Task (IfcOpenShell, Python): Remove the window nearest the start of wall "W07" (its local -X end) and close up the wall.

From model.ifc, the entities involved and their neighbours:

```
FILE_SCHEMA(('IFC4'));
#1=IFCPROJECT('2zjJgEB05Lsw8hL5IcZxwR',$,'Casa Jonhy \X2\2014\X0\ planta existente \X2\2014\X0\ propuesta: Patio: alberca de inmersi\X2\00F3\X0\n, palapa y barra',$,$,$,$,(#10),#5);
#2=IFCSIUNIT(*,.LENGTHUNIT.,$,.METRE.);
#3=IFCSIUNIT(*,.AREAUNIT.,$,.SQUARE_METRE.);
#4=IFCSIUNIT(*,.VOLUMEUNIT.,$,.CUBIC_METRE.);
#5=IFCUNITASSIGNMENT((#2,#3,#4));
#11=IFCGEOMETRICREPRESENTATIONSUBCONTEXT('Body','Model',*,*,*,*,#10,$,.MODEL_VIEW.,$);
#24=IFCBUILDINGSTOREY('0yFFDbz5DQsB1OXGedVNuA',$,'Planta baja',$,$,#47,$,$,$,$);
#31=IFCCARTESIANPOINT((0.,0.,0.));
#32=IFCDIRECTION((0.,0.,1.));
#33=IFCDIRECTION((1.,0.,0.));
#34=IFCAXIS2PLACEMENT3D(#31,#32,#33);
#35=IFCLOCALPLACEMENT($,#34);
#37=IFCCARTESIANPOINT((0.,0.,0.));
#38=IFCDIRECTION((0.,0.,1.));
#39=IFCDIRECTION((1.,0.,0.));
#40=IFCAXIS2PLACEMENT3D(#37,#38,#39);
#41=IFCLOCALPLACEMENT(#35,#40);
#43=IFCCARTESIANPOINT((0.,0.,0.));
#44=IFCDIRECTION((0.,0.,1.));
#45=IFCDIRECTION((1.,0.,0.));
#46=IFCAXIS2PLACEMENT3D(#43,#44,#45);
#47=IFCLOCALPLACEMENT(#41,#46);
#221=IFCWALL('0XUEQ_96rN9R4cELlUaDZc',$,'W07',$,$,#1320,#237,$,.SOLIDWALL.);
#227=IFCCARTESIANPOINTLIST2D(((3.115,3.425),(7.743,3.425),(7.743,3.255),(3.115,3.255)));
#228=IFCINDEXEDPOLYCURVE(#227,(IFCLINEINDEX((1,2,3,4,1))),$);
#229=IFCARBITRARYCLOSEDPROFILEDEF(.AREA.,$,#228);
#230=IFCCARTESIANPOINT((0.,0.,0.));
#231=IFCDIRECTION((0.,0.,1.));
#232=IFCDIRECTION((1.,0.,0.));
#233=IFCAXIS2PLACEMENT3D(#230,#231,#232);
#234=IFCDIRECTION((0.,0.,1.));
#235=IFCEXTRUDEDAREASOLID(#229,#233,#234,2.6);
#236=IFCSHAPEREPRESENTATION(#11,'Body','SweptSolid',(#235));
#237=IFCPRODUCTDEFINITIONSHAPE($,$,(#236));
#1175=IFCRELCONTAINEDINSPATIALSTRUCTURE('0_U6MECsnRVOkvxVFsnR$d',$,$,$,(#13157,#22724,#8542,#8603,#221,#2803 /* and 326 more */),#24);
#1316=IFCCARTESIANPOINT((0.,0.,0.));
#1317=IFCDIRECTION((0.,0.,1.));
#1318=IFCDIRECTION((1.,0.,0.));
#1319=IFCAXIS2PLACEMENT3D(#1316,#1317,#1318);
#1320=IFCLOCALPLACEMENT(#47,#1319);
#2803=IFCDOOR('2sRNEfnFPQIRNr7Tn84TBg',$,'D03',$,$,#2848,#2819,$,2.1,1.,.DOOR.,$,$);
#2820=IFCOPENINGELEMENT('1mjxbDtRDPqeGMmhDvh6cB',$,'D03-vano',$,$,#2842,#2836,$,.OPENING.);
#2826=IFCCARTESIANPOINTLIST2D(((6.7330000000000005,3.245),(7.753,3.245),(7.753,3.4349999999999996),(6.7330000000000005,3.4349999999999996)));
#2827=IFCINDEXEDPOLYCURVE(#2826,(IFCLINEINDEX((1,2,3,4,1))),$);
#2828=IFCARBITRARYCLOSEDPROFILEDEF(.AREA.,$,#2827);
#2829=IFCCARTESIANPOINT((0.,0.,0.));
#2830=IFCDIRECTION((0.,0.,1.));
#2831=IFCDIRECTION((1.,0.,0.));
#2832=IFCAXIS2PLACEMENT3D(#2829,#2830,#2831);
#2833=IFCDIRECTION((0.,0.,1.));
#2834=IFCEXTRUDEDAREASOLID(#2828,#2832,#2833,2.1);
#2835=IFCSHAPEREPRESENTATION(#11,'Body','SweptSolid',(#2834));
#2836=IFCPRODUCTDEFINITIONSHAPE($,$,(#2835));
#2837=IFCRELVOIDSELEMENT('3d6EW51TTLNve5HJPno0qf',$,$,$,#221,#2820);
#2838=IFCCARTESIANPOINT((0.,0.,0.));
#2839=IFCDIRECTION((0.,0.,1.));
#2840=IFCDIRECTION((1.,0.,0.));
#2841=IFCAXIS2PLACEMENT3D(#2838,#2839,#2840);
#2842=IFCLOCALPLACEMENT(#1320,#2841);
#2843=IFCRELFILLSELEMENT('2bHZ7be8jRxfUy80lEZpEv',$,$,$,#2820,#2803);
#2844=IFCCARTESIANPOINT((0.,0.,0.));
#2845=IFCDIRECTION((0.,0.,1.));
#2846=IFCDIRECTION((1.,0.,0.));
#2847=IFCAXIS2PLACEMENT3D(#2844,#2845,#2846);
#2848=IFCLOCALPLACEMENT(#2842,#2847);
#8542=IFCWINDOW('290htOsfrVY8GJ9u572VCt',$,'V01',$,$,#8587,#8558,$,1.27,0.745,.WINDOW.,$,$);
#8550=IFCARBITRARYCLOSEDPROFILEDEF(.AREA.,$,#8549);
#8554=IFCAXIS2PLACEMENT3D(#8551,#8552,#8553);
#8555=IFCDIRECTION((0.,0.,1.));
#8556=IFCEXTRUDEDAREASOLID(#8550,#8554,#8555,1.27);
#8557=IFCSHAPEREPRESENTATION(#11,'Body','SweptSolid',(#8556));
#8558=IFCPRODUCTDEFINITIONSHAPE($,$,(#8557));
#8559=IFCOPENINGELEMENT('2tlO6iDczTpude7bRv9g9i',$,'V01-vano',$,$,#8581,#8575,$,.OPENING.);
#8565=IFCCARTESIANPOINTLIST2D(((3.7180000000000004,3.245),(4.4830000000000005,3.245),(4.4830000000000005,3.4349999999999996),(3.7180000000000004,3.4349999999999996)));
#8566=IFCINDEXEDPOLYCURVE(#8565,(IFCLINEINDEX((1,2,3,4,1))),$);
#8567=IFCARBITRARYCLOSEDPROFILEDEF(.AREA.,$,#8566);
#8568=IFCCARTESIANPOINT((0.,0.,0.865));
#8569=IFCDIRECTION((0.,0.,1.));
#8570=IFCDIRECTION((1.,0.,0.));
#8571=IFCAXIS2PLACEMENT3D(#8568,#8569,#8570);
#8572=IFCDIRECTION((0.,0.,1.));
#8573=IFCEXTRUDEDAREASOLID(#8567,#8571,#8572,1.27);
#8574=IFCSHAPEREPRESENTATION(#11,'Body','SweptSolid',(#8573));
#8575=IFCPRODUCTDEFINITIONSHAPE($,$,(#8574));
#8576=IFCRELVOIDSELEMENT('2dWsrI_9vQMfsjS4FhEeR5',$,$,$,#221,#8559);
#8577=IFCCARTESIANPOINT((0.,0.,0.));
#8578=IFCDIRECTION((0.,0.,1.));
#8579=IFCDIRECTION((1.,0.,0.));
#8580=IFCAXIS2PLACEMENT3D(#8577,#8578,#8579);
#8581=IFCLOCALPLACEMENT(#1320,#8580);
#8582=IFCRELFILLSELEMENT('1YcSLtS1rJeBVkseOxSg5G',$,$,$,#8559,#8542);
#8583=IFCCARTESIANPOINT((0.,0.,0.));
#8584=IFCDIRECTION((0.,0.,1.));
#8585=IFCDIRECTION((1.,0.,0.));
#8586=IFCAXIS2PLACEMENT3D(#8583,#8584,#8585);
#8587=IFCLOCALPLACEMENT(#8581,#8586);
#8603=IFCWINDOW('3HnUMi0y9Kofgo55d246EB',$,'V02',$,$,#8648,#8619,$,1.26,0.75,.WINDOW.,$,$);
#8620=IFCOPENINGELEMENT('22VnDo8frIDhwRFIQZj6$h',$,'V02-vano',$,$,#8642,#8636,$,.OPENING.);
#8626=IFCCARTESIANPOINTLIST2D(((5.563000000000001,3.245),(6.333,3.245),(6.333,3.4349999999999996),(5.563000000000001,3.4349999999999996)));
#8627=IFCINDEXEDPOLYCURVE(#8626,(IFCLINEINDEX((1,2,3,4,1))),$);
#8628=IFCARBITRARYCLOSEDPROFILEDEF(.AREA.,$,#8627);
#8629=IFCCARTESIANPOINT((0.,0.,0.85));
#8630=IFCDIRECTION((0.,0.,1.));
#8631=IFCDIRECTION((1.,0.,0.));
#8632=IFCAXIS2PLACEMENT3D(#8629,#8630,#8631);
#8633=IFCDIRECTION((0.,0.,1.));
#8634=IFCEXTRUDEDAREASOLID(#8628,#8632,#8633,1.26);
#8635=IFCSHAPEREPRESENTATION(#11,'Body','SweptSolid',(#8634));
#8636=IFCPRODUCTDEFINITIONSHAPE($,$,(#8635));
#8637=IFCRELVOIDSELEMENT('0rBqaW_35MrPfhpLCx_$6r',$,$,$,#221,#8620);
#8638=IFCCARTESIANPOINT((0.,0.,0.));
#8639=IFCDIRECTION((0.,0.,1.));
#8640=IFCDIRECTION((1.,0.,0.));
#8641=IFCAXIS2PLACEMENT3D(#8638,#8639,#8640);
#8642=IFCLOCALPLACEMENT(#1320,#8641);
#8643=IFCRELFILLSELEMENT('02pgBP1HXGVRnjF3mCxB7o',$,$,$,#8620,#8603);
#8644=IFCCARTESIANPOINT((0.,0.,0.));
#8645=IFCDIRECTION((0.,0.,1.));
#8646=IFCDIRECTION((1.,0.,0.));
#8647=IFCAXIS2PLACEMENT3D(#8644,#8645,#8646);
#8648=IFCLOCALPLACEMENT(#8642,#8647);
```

```python
import ifcopenshell
import ifcopenshell.api.feature
import ifcopenshell.api.root
import ifcopenshell.geom
import ifcopenshell.util.shape

model = ifcopenshell.open("model.ifc")
settings = ifcopenshell.geom.settings()


def volume(element):
    """Net volume in cubic metres, openings subtracted."""
    shape = ifcopenshell.geom.create_shape(settings, element)
    return ifcopenshell.util.shape.get_volume(shape.geometry)


window = model.by_guid("290htOsfrVY8GJ9u572VCt")
opening = window.FillsVoids[0].RelatingOpeningElement
wall = opening.VoidsElements[0].RelatingBuildingElement
before = volume(wall)

ifcopenshell.api.root.remove_product(model, product=window)
ifcopenshell.api.feature.remove_feature(model, feature=opening)

after = volume(wall)

print(f"wall volume {before:.3f} -> {after:.3f} m3")

model.write("model_edited.ifc")
```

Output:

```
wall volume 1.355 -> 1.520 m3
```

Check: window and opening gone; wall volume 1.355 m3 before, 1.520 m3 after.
